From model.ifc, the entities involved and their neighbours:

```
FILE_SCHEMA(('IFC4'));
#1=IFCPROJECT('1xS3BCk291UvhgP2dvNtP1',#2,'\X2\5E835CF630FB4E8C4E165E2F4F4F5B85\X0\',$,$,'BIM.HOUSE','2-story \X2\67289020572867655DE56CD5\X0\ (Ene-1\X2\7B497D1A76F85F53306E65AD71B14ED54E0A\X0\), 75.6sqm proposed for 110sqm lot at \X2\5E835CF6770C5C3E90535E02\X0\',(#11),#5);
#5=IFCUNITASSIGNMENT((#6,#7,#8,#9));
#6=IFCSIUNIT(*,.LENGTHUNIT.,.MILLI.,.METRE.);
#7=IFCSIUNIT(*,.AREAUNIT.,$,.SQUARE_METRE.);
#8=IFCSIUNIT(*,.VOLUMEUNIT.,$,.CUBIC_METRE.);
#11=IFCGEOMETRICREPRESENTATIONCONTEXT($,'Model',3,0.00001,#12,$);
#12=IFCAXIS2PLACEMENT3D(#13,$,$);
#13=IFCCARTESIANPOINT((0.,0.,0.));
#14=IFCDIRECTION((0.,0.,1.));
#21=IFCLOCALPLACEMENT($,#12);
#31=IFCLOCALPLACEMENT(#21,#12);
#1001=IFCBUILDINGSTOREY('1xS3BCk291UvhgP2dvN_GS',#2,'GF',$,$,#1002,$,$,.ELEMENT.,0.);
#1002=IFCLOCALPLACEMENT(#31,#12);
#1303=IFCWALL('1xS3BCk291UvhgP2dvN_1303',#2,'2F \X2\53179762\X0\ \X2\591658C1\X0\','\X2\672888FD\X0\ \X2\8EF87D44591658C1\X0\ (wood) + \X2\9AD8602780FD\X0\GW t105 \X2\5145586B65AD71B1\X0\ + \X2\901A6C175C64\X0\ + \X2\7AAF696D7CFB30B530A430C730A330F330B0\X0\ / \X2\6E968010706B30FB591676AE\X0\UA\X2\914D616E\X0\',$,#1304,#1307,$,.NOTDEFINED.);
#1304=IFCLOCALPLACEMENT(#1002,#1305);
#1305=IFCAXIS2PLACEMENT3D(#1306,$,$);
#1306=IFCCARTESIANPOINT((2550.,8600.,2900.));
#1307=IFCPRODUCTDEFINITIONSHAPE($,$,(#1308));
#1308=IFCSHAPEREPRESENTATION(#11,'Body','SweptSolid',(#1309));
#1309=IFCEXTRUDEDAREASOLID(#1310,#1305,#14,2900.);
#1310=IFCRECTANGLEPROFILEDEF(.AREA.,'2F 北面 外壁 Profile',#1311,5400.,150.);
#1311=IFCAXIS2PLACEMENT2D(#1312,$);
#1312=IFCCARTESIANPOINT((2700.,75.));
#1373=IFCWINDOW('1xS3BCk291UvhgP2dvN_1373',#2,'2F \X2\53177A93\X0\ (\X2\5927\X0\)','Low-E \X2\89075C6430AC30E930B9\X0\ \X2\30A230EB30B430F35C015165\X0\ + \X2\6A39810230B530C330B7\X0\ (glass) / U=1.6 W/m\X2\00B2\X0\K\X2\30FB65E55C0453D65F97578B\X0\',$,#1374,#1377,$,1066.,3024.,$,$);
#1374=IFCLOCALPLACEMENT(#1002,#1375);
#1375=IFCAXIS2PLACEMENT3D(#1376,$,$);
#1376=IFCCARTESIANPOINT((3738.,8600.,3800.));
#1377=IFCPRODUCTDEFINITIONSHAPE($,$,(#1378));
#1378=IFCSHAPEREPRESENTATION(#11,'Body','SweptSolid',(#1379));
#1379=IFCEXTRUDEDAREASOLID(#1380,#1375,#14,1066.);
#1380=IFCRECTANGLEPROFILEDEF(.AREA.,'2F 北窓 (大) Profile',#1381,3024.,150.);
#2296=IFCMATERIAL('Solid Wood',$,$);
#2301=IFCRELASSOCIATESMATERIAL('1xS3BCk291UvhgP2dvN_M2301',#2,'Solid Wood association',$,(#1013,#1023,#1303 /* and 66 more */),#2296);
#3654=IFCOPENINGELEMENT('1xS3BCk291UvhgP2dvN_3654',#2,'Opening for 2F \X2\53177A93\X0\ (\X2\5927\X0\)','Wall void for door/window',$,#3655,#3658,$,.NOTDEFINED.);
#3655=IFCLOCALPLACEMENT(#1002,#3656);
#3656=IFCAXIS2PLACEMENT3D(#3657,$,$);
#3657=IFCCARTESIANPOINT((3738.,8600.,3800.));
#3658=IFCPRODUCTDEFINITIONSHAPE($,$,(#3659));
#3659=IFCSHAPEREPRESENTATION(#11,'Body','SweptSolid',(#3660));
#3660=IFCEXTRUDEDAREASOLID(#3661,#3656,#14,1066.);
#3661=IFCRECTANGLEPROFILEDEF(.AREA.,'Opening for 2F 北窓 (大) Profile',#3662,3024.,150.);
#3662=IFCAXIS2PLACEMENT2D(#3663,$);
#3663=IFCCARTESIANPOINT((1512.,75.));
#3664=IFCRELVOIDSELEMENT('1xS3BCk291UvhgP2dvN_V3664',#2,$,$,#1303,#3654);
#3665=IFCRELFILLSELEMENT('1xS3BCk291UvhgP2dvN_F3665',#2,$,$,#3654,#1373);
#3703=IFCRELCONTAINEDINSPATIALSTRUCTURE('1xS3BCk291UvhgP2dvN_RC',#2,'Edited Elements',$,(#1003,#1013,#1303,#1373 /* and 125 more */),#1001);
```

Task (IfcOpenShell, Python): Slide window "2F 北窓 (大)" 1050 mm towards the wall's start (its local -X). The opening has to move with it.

```python
import ifcopenshell
import ifcopenshell.api.geometry
import ifcopenshell.util.placement
import ifcopenshell.util.unit

model = ifcopenshell.open("model.ifc")
unit_scale = ifcopenshell.util.unit.calculate_unit_scale(model)

window = model.by_guid("1xS3BCk291UvhgP2dvN_1373")
opening = window.FillsVoids[0].RelatingOpeningElement
wall = opening.VoidsElements[0].RelatingBuildingElement

wall_matrix = ifcopenshell.util.placement.get_local_placement(wall.ObjectPlacement)
shift = wall_matrix[:3, 0] * -1.05 / unit_scale
before = ifcopenshell.util.placement.get_local_placement(window.ObjectPlacement)[:3, 3].copy()

# The window is not placed relative to its opening, so move both.
for product in (opening, window):
    matrix = ifcopenshell.util.placement.get_local_placement(product.ObjectPlacement)
    matrix[:3, 3] += shift
    ifcopenshell.api.geometry.edit_object_placement(model, product=product, matrix=matrix, is_si=False)

after = ifcopenshell.util.placement.get_local_placement(window.ObjectPlacement)[:3, 3]
print("window moved by", (after - before).round(3) + 0.0)

model.write("model_edited.ifc")
```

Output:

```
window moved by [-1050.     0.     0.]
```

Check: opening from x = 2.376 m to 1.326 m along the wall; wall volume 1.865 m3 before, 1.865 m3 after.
